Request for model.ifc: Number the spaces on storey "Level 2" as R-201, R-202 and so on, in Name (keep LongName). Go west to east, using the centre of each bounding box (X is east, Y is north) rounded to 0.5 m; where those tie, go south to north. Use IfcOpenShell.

First a look at what the model holds.

```python
import ifcopenshell
import ifcopenshell.util.element
import ifcopenshell.util.placement

model = ifcopenshell.open("model.ifc")
print(model.schema)
storey = next(s for s in model.by_type("IfcBuildingStorey") if s.Name == "Level 2")
spaces = [e for e in ifcopenshell.util.element.get_decomposition(storey) if e.is_a("IfcSpace")]
for e in sorted(spaces, key=lambda e: e.id()):
    origin = ifcopenshell.util.placement.get_local_placement(e.ObjectPlacement)[:3, 3]
    print(e.id(), e.Name, e.LongName, origin.round(2) + 0.0, sep=" | ")
```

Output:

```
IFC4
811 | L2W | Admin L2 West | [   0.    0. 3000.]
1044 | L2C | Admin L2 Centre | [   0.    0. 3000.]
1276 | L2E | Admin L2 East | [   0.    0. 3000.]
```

```python
import ifcopenshell
import ifcopenshell.geom
import ifcopenshell.util.element
import ifcopenshell.util.shape

model = ifcopenshell.open("model.ifc")
settings = ifcopenshell.geom.settings()
settings.set("use-world-coords", True)


def centre(element):
    shape = ifcopenshell.geom.create_shape(settings, element)
    return ifcopenshell.util.shape.get_bbox_centroid(shape.geometry)


storey = next(s for s in model.by_type("IfcBuildingStorey") if s.Name == "Level 2")
spaces = [e for e in ifcopenshell.util.element.get_decomposition(storey) if e.is_a("IfcSpace")]

# Insertion points can sit at a corner or the storey origin, so sort by the geometry (in metres).
centres = {e: centre(e) for e in spaces}
spaces.sort(key=lambda e: (round(centres[e][0] / 0.5), centres[e][1]))

for i, e in enumerate(spaces, start=1):
    number = f"R-2{i:02d}"
    e.Name = number
    print(e.id(), number)

model.write("model_updated.ifc")
```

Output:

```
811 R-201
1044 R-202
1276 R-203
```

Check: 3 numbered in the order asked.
